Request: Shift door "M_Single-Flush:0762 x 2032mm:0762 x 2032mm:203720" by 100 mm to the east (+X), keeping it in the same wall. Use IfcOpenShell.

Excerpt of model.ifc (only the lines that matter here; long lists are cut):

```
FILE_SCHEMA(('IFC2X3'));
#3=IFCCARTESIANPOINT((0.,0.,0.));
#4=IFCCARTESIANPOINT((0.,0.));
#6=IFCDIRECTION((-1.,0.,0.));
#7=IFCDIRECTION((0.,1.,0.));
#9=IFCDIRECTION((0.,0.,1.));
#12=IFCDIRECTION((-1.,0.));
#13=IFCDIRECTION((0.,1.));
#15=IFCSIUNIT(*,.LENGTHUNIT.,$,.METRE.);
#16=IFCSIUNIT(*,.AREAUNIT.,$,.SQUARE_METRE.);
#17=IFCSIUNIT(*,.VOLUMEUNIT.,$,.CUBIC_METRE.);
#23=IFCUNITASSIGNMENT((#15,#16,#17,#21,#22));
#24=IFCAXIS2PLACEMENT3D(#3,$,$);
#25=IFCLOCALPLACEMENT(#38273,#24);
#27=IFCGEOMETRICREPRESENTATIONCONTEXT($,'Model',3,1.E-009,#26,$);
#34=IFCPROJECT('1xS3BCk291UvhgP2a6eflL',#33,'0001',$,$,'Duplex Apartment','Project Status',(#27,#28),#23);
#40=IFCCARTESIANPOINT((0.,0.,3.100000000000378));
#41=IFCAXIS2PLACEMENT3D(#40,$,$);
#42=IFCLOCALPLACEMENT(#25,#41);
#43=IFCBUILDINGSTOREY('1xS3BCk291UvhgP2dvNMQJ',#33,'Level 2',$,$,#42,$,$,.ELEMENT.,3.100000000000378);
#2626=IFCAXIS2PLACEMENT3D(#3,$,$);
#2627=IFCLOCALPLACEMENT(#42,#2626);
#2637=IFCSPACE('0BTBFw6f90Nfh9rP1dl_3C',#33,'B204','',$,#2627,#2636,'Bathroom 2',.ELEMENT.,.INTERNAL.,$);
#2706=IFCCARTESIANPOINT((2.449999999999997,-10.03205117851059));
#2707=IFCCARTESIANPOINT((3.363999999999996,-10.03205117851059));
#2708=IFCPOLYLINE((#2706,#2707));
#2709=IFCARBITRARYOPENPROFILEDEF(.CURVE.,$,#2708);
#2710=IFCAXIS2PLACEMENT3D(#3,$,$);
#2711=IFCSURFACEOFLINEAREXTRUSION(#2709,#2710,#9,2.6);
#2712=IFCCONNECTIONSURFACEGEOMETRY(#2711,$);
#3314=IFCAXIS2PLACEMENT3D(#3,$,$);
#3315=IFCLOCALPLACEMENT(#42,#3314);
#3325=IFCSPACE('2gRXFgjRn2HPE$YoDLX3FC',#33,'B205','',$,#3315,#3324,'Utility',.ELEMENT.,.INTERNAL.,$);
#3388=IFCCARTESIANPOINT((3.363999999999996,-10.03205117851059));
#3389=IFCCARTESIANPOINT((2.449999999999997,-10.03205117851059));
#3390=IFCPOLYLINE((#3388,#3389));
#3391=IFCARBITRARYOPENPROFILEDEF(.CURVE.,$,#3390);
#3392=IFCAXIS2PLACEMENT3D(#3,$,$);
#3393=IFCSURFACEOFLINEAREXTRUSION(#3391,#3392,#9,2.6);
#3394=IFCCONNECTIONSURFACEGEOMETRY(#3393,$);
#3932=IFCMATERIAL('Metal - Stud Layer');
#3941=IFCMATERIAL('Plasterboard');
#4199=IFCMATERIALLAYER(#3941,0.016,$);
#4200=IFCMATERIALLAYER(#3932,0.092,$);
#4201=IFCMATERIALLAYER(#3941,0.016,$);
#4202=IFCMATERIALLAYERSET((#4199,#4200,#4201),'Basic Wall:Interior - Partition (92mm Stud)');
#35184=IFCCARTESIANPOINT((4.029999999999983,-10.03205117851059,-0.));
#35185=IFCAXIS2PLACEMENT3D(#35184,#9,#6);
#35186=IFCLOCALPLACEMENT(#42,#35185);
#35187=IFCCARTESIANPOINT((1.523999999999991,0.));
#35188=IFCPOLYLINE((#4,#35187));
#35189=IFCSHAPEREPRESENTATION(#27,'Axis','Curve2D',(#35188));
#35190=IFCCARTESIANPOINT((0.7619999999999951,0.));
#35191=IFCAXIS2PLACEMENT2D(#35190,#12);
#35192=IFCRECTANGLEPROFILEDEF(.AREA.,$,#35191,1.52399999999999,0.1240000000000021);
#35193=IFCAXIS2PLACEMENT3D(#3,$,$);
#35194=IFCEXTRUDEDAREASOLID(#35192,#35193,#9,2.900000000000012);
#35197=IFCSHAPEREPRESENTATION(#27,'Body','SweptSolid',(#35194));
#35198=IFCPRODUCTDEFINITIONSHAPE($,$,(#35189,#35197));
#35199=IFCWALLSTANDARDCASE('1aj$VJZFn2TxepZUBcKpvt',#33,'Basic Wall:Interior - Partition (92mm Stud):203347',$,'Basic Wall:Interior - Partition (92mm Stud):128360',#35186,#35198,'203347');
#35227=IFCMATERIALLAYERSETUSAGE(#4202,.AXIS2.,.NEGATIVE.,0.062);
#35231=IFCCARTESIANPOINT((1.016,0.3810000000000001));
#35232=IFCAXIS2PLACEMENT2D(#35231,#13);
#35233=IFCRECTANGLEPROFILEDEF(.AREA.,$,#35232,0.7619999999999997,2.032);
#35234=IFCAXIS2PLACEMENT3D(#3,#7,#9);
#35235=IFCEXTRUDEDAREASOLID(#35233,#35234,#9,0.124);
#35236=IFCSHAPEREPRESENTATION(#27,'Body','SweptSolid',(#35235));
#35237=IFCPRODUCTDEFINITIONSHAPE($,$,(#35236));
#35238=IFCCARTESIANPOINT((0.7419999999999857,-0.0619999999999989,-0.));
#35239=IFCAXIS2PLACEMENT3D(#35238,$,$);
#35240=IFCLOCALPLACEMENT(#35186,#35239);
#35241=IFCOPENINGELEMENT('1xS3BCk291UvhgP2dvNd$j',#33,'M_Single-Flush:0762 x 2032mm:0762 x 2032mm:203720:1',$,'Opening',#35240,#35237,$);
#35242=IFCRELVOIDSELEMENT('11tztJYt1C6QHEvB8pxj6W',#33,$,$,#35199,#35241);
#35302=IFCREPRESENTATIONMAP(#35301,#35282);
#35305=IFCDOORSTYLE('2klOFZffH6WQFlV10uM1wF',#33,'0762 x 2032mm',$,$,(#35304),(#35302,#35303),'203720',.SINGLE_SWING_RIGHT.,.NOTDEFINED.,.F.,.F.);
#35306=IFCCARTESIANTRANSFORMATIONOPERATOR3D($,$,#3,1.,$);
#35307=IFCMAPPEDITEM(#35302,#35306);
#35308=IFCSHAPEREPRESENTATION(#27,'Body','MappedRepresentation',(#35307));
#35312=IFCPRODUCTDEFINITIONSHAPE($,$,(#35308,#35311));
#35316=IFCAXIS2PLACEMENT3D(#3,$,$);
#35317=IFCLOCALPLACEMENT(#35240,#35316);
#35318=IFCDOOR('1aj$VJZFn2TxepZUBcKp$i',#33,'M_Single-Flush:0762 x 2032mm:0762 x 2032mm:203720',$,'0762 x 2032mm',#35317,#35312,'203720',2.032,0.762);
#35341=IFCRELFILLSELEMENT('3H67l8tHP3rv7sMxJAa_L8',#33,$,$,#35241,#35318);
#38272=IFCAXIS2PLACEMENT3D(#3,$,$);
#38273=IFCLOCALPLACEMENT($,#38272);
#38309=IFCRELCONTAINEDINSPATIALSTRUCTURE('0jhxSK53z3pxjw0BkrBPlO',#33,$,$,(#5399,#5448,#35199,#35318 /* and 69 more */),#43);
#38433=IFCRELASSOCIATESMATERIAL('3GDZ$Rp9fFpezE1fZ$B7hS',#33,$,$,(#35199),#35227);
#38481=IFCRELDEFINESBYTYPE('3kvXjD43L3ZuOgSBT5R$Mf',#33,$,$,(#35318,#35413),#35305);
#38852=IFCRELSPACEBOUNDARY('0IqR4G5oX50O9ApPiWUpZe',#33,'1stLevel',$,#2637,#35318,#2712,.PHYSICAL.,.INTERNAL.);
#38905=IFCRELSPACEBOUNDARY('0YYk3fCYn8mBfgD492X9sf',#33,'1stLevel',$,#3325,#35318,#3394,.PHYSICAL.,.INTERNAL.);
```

```python
import numpy as np
import ifcopenshell
import ifcopenshell.api.geometry
import ifcopenshell.util.placement
import ifcopenshell.util.unit

model = ifcopenshell.open("model.ifc")
unit_scale = ifcopenshell.util.unit.calculate_unit_scale(model)

door = model.by_guid("1aj$VJZFn2TxepZUBcKp$i")
opening = door.FillsVoids[0].RelatingOpeningElement
wall = opening.VoidsElements[0].RelatingBuildingElement

wall_matrix = ifcopenshell.util.placement.get_local_placement(wall.ObjectPlacement)
shift = wall_matrix[:3, 0] * -0.1 / unit_scale
before = ifcopenshell.util.placement.get_local_placement(door.ObjectPlacement)[:3, 3].copy()

# The door is placed relative to its opening, so it follows when the opening moves.
matrix = ifcopenshell.util.placement.get_local_placement(opening.ObjectPlacement)
matrix[:3, 3] += shift
ifcopenshell.api.geometry.edit_object_placement(
    model, product=opening, matrix=matrix, is_si=False, should_transform_children=True
)

# Space boundary surfaces are stored in each space's coordinates; move them too.
for rel in door.ProvidesBoundaries:
    if not rel.ConnectionGeometry:
        continue
    surface = rel.ConnectionGeometry.SurfaceOnRelatingElement
    space_matrix = ifcopenshell.util.placement.get_local_placement(rel.RelatingSpace.ObjectPlacement)
    point = np.array(surface.Position.Location.Coordinates) + space_matrix[:3, :3].T @ shift
    surface.Position = model.createIfcAxis2Placement3D(
        model.createIfcCartesianPoint(point.tolist()), surface.Position.Axis, surface.Position.RefDirection
    )

after = ifcopenshell.util.placement.get_local_placement(door.ObjectPlacement)[:3, 3]
print("door moved by", (after - before).round(3) + 0.0)

model.write("model_rev.ifc")
```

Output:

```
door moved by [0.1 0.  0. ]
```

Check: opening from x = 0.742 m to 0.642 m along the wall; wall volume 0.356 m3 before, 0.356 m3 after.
